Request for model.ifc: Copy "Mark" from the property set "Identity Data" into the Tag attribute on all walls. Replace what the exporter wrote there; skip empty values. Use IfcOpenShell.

First a look at what the model holds.

```python
import ifcopenshell
import ifcopenshell.util.element

model = ifcopenshell.open("model.ifc")
print(model.schema)
walls = model.by_type("IfcWall")
print(len(walls), "walls")
for e in walls[:8]:
    source = ifcopenshell.util.element.get_pset(e, "Identity Data", "Mark")
    target = e.Tag
    print(e.id(), repr(source), repr(target), sep=" | ")
```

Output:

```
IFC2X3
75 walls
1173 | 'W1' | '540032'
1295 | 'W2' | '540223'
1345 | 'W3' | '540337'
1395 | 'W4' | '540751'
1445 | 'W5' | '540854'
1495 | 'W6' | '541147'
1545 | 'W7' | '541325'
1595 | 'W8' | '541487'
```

```python
import ifcopenshell
import ifcopenshell.util.element

model = ifcopenshell.open("model.ifc")

count = 0
for e in model.by_type("IfcWall"):
    value = ifcopenshell.util.element.get_pset(e, "Identity Data", "Mark")
    current = e.Tag
    if not value or not value.strip() or current == value:
        continue
    e.Tag = value
    count += 1

print(count, "walls updated")

model.write("model_v2.ifc")
```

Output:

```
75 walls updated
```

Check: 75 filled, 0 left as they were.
